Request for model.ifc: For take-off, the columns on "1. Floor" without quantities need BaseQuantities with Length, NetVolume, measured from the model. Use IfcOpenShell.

First a look at what the model holds.

```python
import ifcopenshell
import ifcopenshell.util.element
import ifcopenshell.util.unit

model = ifcopenshell.open("model.ifc")
print(model.schema)
for unit_type in ("LENGTHUNIT", "AREAUNIT", "VOLUMEUNIT"):
    print(unit_type, ifcopenshell.util.unit.calculate_unit_scale(model, unit_type))
storey = next(s for s in model.by_type("IfcBuildingStorey") if s.Name == "1. Floor")
columns = [e for e in ifcopenshell.util.element.get_decomposition(storey) if e.is_a("IfcColumn")]
for e in sorted(columns, key=lambda e: e.id()):
    print(e.id(), e.is_a(), e.Name, list(ifcopenshell.util.element.get_psets(e, qtos_only=True)), sep=" | ")
```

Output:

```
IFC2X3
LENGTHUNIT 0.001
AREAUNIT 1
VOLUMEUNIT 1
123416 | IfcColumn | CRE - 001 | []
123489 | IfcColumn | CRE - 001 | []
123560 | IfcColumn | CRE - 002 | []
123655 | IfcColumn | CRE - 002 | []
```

```python
import ifcopenshell
import ifcopenshell.api.pset
import ifcopenshell.geom
import ifcopenshell.util.element
import ifcopenshell.util.shape
import ifcopenshell.util.unit

model = ifcopenshell.open("model.ifc")
unit_scale = ifcopenshell.util.unit.calculate_unit_scale(model)
volume_scale = ifcopenshell.util.unit.calculate_unit_scale(model, "VOLUMEUNIT")
settings = ifcopenshell.geom.settings()

storey = next(s for s in model.by_type("IfcBuildingStorey") if s.Name == "1. Floor")
columns = [e for e in ifcopenshell.util.element.get_decomposition(storey) if e.is_a("IfcColumn")]

for e in sorted(columns, key=lambda e: e.id()):
    if ifcopenshell.util.element.get_psets(e, qtos_only=True, should_inherit=False):
        continue
    # Geometry comes back in metres, in the element's own axes.
    shape = ifcopenshell.geom.create_shape(settings, e)
    values = {
        "Length": ifcopenshell.util.shape.get_z(shape.geometry) / unit_scale,
        "NetVolume": ifcopenshell.util.shape.get_volume(shape.geometry) / volume_scale,
    }
    qto = ifcopenshell.api.pset.add_qto(model, product=e, name="BaseQuantities")
    ifcopenshell.api.pset.edit_qto(model, qto=qto, properties=values)
    print(e.id(), {k: round(v, 3) for k, v in values.items()})

model.write("model_rev.ifc")
```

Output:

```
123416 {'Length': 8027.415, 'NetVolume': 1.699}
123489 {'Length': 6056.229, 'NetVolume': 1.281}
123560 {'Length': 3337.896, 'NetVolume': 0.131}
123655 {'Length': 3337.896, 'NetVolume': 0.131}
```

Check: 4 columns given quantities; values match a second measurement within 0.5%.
